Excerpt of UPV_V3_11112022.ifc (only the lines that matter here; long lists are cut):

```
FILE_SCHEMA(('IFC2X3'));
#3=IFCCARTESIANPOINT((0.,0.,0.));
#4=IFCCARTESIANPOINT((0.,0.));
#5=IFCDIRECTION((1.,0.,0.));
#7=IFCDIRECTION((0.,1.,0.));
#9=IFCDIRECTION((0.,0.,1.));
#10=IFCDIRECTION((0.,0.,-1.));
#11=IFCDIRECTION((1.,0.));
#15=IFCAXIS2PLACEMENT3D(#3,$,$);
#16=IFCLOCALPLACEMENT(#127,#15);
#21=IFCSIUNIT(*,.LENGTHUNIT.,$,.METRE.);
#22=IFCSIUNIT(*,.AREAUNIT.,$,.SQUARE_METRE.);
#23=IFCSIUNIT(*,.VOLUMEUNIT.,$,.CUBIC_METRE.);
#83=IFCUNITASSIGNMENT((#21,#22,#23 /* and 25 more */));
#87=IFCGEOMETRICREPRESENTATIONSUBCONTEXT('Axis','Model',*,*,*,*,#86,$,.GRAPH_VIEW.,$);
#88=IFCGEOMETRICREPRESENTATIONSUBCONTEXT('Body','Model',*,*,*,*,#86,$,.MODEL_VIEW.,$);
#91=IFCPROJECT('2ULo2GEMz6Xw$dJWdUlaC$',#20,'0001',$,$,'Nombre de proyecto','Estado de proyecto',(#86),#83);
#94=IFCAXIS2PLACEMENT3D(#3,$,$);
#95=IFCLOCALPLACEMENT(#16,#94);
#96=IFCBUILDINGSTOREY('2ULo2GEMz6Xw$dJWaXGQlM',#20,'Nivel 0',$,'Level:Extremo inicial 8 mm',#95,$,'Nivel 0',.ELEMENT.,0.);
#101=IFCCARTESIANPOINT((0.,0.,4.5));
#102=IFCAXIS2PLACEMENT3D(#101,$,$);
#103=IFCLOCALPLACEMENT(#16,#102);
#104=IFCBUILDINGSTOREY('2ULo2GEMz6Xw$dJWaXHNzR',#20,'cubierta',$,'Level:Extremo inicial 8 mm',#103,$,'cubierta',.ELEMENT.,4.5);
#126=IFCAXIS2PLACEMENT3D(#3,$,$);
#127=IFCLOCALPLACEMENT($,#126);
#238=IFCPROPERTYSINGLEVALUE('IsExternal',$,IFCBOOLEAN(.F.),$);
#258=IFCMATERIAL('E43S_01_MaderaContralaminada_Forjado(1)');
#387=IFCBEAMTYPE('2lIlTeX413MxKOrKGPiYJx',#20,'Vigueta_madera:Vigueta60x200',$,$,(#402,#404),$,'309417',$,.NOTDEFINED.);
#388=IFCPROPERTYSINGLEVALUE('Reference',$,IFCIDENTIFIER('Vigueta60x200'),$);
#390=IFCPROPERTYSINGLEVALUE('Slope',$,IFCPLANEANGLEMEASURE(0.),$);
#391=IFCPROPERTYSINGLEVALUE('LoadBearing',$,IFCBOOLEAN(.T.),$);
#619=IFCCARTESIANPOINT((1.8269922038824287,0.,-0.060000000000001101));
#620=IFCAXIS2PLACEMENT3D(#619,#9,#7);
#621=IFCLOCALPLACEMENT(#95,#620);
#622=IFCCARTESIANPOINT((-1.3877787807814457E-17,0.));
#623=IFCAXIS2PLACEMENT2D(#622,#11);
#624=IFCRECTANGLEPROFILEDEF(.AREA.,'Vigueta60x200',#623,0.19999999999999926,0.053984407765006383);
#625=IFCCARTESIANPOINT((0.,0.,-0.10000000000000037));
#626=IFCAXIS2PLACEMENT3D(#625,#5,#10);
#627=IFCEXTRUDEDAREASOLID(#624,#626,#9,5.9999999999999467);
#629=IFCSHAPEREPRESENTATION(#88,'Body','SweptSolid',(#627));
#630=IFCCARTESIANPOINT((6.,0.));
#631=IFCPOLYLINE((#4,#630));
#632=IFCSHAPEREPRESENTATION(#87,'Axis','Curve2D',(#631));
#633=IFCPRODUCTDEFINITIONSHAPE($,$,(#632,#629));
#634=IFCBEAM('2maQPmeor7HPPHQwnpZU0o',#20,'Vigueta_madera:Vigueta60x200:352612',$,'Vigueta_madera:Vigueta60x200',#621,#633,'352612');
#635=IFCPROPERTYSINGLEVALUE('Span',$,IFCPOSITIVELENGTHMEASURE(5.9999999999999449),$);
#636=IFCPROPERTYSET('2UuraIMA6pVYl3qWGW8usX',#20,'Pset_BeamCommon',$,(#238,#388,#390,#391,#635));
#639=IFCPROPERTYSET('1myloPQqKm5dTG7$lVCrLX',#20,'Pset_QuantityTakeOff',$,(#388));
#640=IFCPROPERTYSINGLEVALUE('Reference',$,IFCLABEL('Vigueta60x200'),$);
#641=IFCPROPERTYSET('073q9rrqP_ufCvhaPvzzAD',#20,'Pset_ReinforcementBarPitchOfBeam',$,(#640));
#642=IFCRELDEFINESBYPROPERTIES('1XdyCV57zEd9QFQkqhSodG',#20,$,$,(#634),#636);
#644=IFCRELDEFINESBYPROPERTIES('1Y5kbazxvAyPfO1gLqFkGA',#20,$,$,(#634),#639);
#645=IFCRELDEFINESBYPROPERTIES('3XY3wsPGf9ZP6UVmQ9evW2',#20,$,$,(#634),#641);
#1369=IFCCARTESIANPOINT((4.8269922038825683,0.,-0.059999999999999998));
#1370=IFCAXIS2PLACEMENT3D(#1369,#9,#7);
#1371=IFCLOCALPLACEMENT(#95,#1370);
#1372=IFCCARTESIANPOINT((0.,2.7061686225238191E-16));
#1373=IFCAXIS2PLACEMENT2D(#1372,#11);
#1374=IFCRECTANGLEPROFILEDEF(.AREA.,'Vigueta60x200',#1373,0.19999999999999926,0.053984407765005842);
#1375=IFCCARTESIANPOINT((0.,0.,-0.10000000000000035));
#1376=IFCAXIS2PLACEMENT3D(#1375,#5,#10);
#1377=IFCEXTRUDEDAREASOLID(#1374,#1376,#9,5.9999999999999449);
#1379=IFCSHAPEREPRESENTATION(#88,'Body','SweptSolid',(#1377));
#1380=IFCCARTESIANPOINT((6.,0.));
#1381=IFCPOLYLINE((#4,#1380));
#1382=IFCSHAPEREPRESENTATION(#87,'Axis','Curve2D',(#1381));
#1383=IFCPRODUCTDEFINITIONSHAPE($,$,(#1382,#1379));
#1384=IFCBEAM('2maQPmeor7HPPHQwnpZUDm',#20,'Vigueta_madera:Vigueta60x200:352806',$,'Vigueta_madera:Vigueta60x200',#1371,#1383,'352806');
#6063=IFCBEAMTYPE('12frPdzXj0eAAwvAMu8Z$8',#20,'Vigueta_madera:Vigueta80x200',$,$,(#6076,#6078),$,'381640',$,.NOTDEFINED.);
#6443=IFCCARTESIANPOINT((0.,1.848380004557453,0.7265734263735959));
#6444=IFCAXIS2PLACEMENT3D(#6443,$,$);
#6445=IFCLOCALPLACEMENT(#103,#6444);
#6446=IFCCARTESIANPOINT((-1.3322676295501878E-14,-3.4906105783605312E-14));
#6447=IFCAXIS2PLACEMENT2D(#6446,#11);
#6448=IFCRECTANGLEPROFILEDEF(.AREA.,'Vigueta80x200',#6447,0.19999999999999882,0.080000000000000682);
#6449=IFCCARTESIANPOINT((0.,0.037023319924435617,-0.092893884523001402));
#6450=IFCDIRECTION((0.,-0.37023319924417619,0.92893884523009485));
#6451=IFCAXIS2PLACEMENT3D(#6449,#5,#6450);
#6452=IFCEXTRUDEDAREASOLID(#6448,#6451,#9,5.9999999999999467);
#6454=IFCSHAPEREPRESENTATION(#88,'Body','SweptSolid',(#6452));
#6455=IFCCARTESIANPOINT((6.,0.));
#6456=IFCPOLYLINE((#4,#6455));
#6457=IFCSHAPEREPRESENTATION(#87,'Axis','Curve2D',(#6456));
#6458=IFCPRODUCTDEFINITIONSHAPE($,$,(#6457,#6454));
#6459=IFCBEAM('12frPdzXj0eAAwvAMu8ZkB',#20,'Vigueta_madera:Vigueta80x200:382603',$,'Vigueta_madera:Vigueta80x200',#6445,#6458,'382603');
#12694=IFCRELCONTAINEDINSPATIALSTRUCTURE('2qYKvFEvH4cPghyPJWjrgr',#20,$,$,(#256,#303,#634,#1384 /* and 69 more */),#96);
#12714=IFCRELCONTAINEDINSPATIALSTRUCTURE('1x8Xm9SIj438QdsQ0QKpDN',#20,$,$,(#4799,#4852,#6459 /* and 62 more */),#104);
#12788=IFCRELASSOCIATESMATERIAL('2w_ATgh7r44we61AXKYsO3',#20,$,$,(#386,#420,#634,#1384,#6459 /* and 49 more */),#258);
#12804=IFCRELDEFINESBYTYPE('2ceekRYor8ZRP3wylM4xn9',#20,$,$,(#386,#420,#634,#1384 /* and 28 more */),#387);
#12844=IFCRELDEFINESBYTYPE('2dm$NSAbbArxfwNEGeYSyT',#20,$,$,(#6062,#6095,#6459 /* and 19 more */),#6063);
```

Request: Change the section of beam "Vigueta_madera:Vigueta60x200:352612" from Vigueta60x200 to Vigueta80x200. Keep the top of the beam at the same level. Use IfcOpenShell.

```python
import ifcopenshell
import ifcopenshell.api.pset
import ifcopenshell.api.type
import ifcopenshell.util.element
import ifcopenshell.util.representation

model = ifcopenshell.open("UPV_V3_11112022.ifc")

member = model.by_guid("2maQPmeor7HPPHQwnpZU0o")
source = next(p for p in model.by_type("IfcRectangleProfileDef") if p.ProfileName == "Vigueta80x200")

body = ifcopenshell.util.representation.get_representation(member, "Model", "Body")
solid = body.Items[0]
old_profile = solid.SweptArea

# Copy the section's sizes but keep this member's own profile position.
profile = ifcopenshell.util.element.copy(model, source)
# Profiles are centred, so shift by half the change in depth to hold the top.
shift = (old_profile.XDim - profile.XDim) / 2
x, y = old_profile.Position.Location.Coordinates
up = (-1.0, 0.0)  # upwards, in the solid's own plane
location = model.createIfcCartesianPoint((x + up[0] * shift, y + up[1] * shift))
profile.Position = model.createIfcAxis2Placement2D(location, old_profile.Position.RefDirection)
solid.SweptArea = profile
if not model.get_total_inverses(old_profile):
    ifcopenshell.util.element.remove_deep2(model, old_profile)

new_type = model.by_id(6063)
ifcopenshell.api.type.assign_type(
    model, related_objects=[member], relating_type=new_type, should_map_representations=False
)
member.Name = member.Name.replace("Vigueta60x200", "Vigueta80x200")
member.ObjectType = "Vigueta_madera:Vigueta80x200"
pset = model.by_id(ifcopenshell.util.element.get_pset(member, "Pset_BeamCommon", should_inherit=False)["id"])
ifcopenshell.api.pset.edit_pset(model, pset=pset, properties={"Reference": "Vigueta80x200"})
pset = model.by_id(ifcopenshell.util.element.get_pset(member, "Pset_QuantityTakeOff", should_inherit=False)["id"])
ifcopenshell.api.pset.edit_pset(model, pset=pset, properties={"Reference": "Vigueta80x200"})
pset = model.by_id(ifcopenshell.util.element.get_pset(member, "Pset_ReinforcementBarPitchOfBeam", should_inherit=False)["id"])
ifcopenshell.api.pset.edit_pset(model, pset=pset, properties={"Reference": "Vigueta80x200"})

print(solid.SweptArea)

model.write("UPV_V3_11112022_edited.ifc")
```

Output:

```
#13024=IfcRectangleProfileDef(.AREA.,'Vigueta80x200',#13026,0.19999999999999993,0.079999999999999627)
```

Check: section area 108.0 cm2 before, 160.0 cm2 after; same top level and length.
